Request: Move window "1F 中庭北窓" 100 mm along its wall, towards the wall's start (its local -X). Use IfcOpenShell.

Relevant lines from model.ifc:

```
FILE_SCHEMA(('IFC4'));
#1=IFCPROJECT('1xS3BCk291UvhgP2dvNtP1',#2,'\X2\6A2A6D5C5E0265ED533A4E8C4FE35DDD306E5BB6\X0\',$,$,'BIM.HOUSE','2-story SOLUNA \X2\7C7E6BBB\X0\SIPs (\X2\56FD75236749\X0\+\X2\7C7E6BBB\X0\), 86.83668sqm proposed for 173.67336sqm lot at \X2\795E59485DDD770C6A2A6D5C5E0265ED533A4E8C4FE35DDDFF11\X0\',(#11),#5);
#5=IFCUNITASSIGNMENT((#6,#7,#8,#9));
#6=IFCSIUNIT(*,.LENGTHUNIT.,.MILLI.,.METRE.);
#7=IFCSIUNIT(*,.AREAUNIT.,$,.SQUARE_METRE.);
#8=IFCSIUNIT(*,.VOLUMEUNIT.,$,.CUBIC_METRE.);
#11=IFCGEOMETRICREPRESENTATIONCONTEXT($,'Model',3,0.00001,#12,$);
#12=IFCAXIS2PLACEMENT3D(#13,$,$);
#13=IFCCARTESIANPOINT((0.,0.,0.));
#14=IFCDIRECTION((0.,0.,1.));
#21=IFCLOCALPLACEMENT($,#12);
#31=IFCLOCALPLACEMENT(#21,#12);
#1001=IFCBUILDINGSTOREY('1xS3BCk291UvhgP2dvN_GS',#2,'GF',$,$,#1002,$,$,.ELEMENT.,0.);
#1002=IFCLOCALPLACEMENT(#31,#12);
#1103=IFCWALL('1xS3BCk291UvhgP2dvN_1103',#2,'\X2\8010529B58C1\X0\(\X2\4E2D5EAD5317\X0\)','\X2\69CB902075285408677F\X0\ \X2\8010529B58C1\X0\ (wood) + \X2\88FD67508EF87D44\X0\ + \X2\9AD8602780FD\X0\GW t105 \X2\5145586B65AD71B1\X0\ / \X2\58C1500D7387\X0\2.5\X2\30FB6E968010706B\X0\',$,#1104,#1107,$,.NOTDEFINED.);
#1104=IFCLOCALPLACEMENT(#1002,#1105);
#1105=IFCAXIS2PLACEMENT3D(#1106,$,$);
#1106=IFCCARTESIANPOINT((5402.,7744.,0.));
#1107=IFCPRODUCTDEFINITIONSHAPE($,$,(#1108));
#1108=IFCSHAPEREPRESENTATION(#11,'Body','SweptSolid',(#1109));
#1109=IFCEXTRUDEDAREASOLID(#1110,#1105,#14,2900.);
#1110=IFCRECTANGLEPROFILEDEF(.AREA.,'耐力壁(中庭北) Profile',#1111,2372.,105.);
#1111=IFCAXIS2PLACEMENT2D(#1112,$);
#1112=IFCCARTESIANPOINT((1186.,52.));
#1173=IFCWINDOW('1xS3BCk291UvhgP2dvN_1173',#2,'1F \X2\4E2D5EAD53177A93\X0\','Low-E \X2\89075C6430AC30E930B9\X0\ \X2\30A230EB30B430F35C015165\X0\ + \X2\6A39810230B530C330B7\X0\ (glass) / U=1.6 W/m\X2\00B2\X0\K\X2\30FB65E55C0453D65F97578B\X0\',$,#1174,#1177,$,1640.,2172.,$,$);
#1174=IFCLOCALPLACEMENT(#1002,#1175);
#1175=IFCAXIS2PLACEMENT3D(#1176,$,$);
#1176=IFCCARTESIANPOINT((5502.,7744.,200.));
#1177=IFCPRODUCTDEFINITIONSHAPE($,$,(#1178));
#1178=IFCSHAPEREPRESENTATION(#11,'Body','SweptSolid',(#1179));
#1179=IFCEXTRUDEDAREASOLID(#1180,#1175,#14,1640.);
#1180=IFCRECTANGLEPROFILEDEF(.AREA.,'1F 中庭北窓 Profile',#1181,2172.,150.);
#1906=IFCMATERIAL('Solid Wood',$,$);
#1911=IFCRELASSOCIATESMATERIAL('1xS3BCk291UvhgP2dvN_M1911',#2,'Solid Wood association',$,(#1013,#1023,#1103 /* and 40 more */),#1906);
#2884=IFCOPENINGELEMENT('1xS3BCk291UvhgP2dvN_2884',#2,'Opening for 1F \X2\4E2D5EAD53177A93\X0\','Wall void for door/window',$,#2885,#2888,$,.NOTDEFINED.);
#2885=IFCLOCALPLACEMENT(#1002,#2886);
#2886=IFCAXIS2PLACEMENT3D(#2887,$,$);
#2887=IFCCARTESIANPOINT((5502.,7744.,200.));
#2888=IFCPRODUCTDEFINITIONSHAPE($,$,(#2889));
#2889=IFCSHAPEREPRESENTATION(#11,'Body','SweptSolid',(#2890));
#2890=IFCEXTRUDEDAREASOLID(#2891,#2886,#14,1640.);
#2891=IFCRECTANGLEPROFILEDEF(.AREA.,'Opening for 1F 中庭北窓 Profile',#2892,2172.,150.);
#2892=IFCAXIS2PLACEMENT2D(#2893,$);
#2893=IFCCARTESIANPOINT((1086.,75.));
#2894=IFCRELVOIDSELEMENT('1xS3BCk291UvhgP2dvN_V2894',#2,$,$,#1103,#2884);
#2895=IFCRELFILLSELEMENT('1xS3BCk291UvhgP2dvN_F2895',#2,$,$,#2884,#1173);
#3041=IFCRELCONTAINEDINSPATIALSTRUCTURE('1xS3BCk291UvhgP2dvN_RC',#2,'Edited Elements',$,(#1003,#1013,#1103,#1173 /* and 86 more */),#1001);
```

```python
import ifcopenshell
import ifcopenshell.api.geometry
import ifcopenshell.util.placement
import ifcopenshell.util.unit

model = ifcopenshell.open("model.ifc")
unit_scale = ifcopenshell.util.unit.calculate_unit_scale(model)

window = model.by_guid("1xS3BCk291UvhgP2dvN_1173")
opening = window.FillsVoids[0].RelatingOpeningElement
wall = opening.VoidsElements[0].RelatingBuildingElement

wall_matrix = ifcopenshell.util.placement.get_local_placement(wall.ObjectPlacement)
shift = wall_matrix[:3, 0] * -0.1 / unit_scale
before = ifcopenshell.util.placement.get_local_placement(window.ObjectPlacement)[:3, 3].copy()

# The window is not placed relative to its opening, so move both.
for product in (opening, window):
    matrix = ifcopenshell.util.placement.get_local_placement(product.ObjectPlacement)
    matrix[:3, 3] += shift
    ifcopenshell.api.geometry.edit_object_placement(model, product=product, matrix=matrix, is_si=False)

after = ifcopenshell.util.placement.get_local_placement(window.ObjectPlacement)[:3, 3]
print("window moved by", (after - before).round(3) + 0.0)

model.write("model_v2.ifc")
```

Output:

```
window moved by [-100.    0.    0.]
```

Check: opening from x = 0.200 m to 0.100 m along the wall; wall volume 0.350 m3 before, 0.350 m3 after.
